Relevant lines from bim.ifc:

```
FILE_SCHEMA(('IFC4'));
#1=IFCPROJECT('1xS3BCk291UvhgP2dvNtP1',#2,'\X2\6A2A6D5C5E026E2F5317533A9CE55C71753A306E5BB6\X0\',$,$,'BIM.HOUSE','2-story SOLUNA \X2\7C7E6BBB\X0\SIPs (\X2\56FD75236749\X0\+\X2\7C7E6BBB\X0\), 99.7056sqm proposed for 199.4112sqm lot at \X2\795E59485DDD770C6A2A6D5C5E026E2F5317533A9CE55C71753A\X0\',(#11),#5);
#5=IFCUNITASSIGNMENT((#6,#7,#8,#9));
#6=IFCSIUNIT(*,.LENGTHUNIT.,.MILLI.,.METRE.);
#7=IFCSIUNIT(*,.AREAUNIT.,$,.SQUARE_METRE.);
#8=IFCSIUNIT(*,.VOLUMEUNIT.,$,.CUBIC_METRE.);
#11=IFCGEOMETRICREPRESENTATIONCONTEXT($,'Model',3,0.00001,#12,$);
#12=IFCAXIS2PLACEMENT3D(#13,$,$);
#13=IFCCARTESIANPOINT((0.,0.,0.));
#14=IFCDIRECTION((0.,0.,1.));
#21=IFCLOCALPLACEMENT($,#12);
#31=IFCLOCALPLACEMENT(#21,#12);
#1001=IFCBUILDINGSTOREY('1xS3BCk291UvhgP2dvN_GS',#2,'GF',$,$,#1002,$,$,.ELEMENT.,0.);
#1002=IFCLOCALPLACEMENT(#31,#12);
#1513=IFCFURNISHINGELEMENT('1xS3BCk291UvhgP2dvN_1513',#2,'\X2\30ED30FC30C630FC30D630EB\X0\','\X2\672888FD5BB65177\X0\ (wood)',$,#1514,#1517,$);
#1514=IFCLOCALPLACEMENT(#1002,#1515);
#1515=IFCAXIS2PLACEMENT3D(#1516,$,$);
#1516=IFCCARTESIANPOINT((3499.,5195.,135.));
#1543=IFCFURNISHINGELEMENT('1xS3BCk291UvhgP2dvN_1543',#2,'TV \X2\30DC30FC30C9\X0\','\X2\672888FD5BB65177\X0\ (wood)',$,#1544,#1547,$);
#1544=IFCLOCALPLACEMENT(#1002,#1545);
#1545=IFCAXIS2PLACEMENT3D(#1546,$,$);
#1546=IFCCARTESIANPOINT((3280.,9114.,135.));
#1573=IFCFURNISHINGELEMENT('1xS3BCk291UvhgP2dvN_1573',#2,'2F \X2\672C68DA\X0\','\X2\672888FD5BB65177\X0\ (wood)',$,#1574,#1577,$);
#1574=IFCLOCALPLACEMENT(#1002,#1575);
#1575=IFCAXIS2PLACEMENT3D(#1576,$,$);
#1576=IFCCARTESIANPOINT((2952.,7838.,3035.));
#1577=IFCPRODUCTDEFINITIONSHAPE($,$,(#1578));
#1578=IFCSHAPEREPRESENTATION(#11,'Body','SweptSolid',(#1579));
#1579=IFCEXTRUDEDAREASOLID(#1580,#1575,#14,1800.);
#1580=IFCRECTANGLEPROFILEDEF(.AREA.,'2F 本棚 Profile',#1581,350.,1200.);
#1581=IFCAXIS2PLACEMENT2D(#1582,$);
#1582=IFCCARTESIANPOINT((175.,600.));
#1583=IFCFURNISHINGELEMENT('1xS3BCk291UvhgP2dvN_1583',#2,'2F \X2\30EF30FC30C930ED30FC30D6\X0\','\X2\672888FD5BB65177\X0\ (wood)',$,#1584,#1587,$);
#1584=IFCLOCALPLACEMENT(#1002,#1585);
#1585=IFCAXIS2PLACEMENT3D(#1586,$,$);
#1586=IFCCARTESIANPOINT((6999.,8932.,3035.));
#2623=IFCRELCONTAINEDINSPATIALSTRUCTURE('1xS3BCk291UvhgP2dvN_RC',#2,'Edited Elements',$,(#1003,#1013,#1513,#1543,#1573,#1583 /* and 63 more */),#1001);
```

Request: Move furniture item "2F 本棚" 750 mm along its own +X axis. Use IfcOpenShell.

```python
import ifcopenshell
import ifcopenshell.api.geometry
import ifcopenshell.util.placement
import ifcopenshell.util.unit

model = ifcopenshell.open("bim.ifc")
unit_scale = ifcopenshell.util.unit.calculate_unit_scale(model)

item = model.by_guid("1xS3BCk291UvhgP2dvN_1573")
matrix = ifcopenshell.util.placement.get_local_placement(item.ObjectPlacement)
matrix[:3, 3] += matrix[:3, 0] * 0.75 / unit_scale
ifcopenshell.api.geometry.edit_object_placement(model, product=item, matrix=matrix, is_si=False)

print(ifcopenshell.util.placement.get_local_placement(item.ObjectPlacement).round(3) + 0.0)

model.write("bim_edited.ifc")
```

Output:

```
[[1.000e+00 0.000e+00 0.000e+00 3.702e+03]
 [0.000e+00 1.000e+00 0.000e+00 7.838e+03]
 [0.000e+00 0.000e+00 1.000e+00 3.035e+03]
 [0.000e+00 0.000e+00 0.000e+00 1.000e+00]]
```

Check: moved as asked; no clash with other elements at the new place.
